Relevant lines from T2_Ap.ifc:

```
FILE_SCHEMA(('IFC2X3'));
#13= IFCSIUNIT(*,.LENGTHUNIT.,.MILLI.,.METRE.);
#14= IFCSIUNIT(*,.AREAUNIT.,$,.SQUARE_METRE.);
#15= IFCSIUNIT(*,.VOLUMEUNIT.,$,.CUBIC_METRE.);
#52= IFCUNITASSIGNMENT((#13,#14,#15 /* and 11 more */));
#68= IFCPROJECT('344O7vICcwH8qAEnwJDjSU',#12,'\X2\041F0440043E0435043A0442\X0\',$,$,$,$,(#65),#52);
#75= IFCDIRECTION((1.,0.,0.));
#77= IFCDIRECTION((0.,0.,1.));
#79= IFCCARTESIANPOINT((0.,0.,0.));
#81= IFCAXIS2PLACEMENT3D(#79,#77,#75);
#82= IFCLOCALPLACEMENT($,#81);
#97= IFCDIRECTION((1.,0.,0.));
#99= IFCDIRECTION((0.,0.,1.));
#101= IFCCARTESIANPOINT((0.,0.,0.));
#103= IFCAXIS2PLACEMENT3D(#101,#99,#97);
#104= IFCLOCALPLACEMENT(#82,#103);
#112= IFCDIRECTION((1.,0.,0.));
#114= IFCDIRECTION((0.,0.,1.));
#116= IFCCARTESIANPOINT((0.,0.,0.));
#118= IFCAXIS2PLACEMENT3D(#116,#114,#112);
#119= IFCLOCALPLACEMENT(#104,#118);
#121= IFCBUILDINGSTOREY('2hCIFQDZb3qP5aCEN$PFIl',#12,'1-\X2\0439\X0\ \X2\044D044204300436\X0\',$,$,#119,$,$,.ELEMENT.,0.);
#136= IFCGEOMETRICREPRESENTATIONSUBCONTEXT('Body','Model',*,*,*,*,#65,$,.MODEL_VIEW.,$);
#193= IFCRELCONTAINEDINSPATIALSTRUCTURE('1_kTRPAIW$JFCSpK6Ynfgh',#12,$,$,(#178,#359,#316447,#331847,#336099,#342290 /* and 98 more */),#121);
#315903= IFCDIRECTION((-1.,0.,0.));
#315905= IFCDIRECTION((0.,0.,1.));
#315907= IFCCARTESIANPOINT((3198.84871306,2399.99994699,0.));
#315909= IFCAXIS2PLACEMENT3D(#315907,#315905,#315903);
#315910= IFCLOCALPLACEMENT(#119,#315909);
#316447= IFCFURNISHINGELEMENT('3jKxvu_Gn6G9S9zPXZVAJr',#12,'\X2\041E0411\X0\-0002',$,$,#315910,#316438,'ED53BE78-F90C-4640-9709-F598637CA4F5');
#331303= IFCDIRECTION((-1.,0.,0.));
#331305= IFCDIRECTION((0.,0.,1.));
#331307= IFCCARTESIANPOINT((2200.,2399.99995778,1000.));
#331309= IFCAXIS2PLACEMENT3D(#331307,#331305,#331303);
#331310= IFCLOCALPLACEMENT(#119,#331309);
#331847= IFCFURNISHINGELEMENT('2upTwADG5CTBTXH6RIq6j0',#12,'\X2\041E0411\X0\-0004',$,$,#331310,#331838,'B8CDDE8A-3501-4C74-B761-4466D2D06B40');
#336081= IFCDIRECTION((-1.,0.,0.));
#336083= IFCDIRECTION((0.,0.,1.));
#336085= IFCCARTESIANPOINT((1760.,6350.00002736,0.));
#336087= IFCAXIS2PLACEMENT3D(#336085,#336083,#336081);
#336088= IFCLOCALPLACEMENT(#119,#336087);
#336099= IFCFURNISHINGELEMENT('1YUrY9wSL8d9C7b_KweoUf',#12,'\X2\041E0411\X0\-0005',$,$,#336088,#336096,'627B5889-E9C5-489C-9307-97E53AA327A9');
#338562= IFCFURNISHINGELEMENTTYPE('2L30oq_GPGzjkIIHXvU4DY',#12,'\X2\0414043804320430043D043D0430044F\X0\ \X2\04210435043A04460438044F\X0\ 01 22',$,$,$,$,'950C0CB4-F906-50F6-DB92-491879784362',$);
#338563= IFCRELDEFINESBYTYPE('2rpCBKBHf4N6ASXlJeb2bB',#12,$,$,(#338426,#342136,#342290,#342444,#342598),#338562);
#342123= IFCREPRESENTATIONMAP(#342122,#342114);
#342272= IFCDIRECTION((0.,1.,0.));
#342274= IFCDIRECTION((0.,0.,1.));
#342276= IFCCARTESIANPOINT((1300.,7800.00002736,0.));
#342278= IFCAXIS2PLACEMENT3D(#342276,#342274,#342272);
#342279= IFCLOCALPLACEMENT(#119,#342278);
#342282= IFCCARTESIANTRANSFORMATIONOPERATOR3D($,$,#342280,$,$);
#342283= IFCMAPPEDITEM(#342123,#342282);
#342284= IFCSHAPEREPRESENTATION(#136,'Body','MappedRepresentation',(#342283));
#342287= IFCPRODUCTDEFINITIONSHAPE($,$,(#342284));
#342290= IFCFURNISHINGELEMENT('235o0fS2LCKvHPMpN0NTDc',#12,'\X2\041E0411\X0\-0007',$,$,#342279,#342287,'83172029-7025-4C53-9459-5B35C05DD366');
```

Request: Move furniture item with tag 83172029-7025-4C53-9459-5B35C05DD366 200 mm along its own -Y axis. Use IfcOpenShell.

```python
import ifcopenshell
import ifcopenshell.api.geometry
import ifcopenshell.util.placement
import ifcopenshell.util.unit

model = ifcopenshell.open("T2_Ap.ifc")
unit_scale = ifcopenshell.util.unit.calculate_unit_scale(model)

item = model.by_id(342290)
matrix = ifcopenshell.util.placement.get_local_placement(item.ObjectPlacement)
matrix[:3, 3] -= matrix[:3, 1] * 0.2 / unit_scale
ifcopenshell.api.geometry.edit_object_placement(model, product=item, matrix=matrix, is_si=False)

print(ifcopenshell.util.placement.get_local_placement(item.ObjectPlacement).round(3) + 0.0)

model.write("T2_Ap_rev.ifc")
```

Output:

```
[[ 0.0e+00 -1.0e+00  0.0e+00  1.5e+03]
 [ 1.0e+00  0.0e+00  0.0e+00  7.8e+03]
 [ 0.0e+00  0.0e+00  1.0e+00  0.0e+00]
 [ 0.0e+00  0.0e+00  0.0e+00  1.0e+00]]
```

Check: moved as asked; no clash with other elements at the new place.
